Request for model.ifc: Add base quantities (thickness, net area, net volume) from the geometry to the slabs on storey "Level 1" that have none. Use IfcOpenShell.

First a look at what the model holds.

```python
import ifcopenshell
import ifcopenshell.util.element
import ifcopenshell.util.unit

model = ifcopenshell.open("model.ifc")
print(model.schema)
for unit_type in ("LENGTHUNIT", "AREAUNIT", "VOLUMEUNIT"):
    print(unit_type, ifcopenshell.util.unit.calculate_unit_scale(model, unit_type))
storey = next(s for s in model.by_type("IfcBuildingStorey") if s.Name == "Level 1")
slabs = [e for e in ifcopenshell.util.element.get_decomposition(storey) if e.is_a("IfcSlab")]
for e in sorted(slabs, key=lambda e: e.id()):
    print(e.id(), e.is_a(), e.Name, list(ifcopenshell.util.element.get_psets(e, qtos_only=True)), sep=" | ")
```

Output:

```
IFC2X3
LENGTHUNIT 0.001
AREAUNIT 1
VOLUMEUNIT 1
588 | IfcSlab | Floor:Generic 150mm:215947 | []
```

```python
import ifcopenshell
import ifcopenshell.api.pset
import ifcopenshell.geom
import ifcopenshell.util.element
import ifcopenshell.util.shape
import ifcopenshell.util.unit

model = ifcopenshell.open("model.ifc")
unit_scale = ifcopenshell.util.unit.calculate_unit_scale(model)
area_scale = ifcopenshell.util.unit.calculate_unit_scale(model, "AREAUNIT")
volume_scale = ifcopenshell.util.unit.calculate_unit_scale(model, "VOLUMEUNIT")
settings = ifcopenshell.geom.settings()

storey = next(s for s in model.by_type("IfcBuildingStorey") if s.Name == "Level 1")
slabs = [e for e in ifcopenshell.util.element.get_decomposition(storey) if e.is_a("IfcSlab")]

for e in sorted(slabs, key=lambda e: e.id()):
    if ifcopenshell.util.element.get_psets(e, qtos_only=True, should_inherit=False):
        continue
    # Geometry comes back in metres, in the element's own axes.
    shape = ifcopenshell.geom.create_shape(settings, e)
    values = {
        "Width": ifcopenshell.util.shape.get_z(shape.geometry) / unit_scale,
        "NetArea": ifcopenshell.util.shape.get_footprint_area(shape.geometry) / area_scale,
        "NetVolume": ifcopenshell.util.shape.get_volume(shape.geometry) / volume_scale,
    }
    qto = ifcopenshell.api.pset.add_qto(model, product=e, name="BaseQuantities")
    ifcopenshell.api.pset.edit_qto(model, qto=qto, properties=values)
    print(e.id(), {k: round(v, 3) for k, v in values.items()})

model.write("model_updated.ifc")
```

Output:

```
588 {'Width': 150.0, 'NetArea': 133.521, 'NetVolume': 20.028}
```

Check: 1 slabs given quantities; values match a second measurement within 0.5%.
